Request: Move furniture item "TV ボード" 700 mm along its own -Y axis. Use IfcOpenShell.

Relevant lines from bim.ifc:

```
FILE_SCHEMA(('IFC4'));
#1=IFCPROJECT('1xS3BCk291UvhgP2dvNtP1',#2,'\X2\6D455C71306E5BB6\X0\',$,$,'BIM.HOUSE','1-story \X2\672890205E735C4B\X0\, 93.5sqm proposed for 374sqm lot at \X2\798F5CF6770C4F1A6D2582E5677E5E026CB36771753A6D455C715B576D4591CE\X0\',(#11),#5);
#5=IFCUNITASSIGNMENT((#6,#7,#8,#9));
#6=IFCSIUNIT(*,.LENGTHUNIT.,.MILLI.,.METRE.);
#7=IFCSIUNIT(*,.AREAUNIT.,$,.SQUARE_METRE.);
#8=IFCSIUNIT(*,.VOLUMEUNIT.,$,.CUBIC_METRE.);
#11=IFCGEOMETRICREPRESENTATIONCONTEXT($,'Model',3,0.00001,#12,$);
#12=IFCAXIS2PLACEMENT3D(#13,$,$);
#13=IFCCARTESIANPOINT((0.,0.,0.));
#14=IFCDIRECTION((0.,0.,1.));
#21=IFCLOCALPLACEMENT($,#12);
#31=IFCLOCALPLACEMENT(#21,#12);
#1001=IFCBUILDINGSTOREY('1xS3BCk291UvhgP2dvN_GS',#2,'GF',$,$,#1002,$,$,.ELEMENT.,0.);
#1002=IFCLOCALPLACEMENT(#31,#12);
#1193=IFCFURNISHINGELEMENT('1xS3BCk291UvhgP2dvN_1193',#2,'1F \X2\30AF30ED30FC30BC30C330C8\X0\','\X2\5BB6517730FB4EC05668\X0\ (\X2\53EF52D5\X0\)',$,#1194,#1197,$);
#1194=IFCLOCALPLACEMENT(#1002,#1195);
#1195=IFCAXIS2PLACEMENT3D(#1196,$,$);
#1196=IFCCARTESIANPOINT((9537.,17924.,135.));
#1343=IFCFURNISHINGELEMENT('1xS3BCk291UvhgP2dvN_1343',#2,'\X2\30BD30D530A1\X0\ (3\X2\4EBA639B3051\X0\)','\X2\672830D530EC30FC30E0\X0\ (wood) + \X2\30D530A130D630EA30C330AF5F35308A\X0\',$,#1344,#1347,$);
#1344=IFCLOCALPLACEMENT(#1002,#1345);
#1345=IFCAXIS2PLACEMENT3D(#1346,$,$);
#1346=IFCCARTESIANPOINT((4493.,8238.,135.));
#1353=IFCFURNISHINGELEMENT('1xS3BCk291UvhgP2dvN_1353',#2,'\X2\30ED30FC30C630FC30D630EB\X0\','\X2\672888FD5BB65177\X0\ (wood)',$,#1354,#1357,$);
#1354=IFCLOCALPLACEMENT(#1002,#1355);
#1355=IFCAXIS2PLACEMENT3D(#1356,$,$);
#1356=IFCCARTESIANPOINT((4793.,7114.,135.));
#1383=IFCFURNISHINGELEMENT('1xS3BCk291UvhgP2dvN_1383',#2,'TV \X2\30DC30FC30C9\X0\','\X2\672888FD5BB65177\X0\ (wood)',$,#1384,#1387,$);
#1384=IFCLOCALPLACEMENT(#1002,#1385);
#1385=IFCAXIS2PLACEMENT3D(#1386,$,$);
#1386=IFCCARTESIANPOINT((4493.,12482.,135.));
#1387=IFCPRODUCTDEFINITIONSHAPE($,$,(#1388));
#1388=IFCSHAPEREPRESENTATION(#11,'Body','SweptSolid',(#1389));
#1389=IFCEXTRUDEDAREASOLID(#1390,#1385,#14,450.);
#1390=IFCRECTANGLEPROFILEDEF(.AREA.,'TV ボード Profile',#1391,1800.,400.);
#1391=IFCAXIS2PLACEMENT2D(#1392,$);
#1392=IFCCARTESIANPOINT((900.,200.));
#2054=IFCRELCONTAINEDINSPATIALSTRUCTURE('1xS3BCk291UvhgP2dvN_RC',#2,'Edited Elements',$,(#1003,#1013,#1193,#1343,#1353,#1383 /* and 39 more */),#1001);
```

```python
import ifcopenshell
import ifcopenshell.api.geometry
import ifcopenshell.util.placement
import ifcopenshell.util.unit

model = ifcopenshell.open("bim.ifc")
unit_scale = ifcopenshell.util.unit.calculate_unit_scale(model)

item = model.by_guid("1xS3BCk291UvhgP2dvN_1383")
matrix = ifcopenshell.util.placement.get_local_placement(item.ObjectPlacement)
matrix[:3, 3] -= matrix[:3, 1] * 0.7 / unit_scale
ifcopenshell.api.geometry.edit_object_placement(model, product=item, matrix=matrix, is_si=False)

print(ifcopenshell.util.placement.get_local_placement(item.ObjectPlacement).round(3) + 0.0)

model.write("bim_updated.ifc")
```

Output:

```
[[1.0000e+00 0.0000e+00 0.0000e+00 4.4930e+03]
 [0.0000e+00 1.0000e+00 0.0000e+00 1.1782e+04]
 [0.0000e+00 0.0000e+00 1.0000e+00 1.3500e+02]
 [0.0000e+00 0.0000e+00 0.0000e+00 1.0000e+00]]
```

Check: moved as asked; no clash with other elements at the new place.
